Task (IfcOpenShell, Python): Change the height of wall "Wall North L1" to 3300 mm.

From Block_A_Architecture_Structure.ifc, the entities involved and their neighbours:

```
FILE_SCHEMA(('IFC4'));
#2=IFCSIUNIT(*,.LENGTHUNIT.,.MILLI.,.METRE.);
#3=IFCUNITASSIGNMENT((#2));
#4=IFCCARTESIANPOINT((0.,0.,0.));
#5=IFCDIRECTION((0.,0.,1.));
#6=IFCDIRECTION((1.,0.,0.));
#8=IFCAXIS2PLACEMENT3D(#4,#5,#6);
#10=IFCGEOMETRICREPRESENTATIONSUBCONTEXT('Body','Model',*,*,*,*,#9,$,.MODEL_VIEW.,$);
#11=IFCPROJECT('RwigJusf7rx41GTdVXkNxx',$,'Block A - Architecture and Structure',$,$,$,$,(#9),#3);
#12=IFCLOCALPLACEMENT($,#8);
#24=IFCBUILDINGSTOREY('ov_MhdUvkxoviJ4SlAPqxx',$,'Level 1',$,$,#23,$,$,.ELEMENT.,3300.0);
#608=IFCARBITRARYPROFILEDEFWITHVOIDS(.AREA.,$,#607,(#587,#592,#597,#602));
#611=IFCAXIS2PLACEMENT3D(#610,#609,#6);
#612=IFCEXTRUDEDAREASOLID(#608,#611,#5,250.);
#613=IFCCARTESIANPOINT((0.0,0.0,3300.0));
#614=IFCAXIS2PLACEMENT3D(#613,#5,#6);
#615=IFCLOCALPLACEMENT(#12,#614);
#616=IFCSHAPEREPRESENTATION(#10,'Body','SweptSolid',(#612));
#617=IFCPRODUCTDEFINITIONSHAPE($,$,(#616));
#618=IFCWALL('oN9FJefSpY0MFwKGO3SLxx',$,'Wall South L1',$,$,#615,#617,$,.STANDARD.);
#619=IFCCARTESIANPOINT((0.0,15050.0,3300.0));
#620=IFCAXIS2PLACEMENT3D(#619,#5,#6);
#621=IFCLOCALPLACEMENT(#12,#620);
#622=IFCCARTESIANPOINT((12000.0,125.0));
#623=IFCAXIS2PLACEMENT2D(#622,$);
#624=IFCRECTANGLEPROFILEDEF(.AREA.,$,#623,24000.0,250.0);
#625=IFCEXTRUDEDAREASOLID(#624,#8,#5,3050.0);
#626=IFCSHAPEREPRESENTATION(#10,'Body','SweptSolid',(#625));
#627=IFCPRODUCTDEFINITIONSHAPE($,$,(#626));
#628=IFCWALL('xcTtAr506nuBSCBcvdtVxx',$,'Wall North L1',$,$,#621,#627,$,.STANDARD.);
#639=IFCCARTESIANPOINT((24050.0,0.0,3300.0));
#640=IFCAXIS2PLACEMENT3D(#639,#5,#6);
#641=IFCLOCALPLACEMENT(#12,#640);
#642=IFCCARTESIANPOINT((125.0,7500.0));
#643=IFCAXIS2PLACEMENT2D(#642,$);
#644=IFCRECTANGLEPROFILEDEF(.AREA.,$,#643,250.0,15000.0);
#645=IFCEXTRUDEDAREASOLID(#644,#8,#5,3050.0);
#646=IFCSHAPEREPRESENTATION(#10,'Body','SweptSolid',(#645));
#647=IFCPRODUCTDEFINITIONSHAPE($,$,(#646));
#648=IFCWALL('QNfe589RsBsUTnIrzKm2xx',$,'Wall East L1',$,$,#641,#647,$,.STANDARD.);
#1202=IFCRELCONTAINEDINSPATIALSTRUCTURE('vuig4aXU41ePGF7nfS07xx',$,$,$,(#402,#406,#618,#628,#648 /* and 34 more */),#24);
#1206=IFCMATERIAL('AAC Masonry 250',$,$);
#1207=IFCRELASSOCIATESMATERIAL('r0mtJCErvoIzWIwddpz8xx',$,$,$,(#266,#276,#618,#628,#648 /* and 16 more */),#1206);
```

```python
import ifcopenshell
import ifcopenshell.geom
import ifcopenshell.util.representation
import ifcopenshell.util.shape
import ifcopenshell.util.unit

model = ifcopenshell.open("Block_A_Architecture_Structure.ifc")
unit_scale = ifcopenshell.util.unit.calculate_unit_scale(model)
settings = ifcopenshell.geom.settings()


def volume(element):
    """Net volume in cubic metres, openings subtracted."""
    shape = ifcopenshell.geom.create_shape(settings, element)
    return ifcopenshell.util.shape.get_volume(shape.geometry)


wall = model.by_guid("xcTtAr506nuBSCBcvdtVxx")
before = volume(wall)

body = ifcopenshell.util.representation.get_representation(wall, "Model", "Body")
solid = body.Items[0]
old_height = solid.Depth
solid.Depth = 3.3 / unit_scale
after = volume(wall)

print(f"height {old_height:g} -> {solid.Depth:g}, volume {before:.3f} -> {after:.3f} m3")

model.write("Block_A_Architecture_Structure_updated.ifc")
```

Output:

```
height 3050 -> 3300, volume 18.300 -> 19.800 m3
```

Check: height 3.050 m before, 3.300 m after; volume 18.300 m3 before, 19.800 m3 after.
